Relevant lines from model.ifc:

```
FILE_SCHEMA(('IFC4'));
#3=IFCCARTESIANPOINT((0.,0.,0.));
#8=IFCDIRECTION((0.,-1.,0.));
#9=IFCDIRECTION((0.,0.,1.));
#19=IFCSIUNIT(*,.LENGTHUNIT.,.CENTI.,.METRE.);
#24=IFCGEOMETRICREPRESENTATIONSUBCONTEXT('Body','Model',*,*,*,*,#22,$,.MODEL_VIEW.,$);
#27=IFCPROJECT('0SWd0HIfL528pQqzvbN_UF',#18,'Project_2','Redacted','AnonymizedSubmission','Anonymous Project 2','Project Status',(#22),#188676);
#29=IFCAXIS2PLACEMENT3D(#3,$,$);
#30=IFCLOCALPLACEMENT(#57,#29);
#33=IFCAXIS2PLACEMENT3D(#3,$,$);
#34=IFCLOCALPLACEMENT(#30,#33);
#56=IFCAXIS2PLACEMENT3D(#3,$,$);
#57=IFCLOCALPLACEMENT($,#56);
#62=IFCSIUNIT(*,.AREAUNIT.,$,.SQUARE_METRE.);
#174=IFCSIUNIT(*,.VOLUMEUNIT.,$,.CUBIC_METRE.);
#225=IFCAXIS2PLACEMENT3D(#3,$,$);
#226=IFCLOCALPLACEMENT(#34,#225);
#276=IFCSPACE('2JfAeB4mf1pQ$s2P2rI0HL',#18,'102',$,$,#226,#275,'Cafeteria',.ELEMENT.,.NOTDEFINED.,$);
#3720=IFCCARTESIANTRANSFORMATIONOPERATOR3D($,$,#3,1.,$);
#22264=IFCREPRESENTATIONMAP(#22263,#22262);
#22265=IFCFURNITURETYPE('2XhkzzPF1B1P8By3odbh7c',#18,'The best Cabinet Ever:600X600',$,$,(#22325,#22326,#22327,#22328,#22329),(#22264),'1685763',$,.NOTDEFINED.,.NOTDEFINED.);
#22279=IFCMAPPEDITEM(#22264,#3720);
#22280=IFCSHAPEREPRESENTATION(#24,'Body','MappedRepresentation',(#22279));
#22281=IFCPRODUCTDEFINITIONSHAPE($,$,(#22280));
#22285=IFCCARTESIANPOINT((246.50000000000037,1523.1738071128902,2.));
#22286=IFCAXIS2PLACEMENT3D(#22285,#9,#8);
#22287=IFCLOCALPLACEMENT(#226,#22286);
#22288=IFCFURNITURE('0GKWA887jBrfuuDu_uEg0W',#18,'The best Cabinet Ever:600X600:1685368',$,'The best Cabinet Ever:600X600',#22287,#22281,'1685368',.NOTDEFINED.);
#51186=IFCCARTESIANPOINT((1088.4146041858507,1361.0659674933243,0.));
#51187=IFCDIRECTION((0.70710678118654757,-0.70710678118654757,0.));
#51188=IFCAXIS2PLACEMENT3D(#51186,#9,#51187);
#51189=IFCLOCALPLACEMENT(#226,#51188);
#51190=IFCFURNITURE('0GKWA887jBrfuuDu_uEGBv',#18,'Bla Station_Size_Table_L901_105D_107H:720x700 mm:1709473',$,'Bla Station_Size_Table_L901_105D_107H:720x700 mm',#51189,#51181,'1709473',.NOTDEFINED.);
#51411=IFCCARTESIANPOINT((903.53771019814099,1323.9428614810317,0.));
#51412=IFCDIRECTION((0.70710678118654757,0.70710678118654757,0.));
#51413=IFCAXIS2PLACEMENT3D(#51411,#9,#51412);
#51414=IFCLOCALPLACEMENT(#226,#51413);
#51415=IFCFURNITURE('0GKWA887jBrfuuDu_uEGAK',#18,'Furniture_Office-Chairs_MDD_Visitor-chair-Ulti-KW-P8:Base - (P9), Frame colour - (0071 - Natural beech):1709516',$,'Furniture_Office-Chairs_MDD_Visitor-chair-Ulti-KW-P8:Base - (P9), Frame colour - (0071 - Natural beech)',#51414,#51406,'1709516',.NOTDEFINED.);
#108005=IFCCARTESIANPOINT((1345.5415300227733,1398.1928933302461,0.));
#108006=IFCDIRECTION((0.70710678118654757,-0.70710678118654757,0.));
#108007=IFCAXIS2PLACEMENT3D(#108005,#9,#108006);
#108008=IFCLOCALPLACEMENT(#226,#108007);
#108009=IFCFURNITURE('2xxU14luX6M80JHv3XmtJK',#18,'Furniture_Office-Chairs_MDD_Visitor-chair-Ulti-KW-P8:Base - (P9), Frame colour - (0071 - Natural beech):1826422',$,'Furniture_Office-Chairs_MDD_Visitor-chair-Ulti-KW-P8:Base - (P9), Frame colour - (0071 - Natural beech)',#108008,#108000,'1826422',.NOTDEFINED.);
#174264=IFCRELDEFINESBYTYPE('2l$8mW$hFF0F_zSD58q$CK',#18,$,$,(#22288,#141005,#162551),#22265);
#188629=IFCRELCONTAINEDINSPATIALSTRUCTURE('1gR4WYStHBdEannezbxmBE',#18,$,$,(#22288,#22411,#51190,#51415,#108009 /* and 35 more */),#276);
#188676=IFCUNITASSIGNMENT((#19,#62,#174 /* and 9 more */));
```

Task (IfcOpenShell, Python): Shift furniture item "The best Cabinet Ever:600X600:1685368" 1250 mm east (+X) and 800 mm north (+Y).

```python
import ifcopenshell
import ifcopenshell.api.geometry
import ifcopenshell.util.placement
import ifcopenshell.util.unit

model = ifcopenshell.open("model.ifc")
unit_scale = ifcopenshell.util.unit.calculate_unit_scale(model)

item = model.by_id(22288)
matrix = ifcopenshell.util.placement.get_local_placement(item.ObjectPlacement)
matrix[0, 3] += 1.25 / unit_scale
matrix[1, 3] += 0.8 / unit_scale
ifcopenshell.api.geometry.edit_object_placement(model, product=item, matrix=matrix, is_si=False)

print(ifcopenshell.util.placement.get_local_placement(item.ObjectPlacement).round(3) + 0.0)

model.write("model_rev.ifc")
```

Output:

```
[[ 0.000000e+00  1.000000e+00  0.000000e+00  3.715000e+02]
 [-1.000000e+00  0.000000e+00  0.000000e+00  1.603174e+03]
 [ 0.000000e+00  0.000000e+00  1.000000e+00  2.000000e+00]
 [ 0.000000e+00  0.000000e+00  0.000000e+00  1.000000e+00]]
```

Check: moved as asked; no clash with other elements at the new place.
